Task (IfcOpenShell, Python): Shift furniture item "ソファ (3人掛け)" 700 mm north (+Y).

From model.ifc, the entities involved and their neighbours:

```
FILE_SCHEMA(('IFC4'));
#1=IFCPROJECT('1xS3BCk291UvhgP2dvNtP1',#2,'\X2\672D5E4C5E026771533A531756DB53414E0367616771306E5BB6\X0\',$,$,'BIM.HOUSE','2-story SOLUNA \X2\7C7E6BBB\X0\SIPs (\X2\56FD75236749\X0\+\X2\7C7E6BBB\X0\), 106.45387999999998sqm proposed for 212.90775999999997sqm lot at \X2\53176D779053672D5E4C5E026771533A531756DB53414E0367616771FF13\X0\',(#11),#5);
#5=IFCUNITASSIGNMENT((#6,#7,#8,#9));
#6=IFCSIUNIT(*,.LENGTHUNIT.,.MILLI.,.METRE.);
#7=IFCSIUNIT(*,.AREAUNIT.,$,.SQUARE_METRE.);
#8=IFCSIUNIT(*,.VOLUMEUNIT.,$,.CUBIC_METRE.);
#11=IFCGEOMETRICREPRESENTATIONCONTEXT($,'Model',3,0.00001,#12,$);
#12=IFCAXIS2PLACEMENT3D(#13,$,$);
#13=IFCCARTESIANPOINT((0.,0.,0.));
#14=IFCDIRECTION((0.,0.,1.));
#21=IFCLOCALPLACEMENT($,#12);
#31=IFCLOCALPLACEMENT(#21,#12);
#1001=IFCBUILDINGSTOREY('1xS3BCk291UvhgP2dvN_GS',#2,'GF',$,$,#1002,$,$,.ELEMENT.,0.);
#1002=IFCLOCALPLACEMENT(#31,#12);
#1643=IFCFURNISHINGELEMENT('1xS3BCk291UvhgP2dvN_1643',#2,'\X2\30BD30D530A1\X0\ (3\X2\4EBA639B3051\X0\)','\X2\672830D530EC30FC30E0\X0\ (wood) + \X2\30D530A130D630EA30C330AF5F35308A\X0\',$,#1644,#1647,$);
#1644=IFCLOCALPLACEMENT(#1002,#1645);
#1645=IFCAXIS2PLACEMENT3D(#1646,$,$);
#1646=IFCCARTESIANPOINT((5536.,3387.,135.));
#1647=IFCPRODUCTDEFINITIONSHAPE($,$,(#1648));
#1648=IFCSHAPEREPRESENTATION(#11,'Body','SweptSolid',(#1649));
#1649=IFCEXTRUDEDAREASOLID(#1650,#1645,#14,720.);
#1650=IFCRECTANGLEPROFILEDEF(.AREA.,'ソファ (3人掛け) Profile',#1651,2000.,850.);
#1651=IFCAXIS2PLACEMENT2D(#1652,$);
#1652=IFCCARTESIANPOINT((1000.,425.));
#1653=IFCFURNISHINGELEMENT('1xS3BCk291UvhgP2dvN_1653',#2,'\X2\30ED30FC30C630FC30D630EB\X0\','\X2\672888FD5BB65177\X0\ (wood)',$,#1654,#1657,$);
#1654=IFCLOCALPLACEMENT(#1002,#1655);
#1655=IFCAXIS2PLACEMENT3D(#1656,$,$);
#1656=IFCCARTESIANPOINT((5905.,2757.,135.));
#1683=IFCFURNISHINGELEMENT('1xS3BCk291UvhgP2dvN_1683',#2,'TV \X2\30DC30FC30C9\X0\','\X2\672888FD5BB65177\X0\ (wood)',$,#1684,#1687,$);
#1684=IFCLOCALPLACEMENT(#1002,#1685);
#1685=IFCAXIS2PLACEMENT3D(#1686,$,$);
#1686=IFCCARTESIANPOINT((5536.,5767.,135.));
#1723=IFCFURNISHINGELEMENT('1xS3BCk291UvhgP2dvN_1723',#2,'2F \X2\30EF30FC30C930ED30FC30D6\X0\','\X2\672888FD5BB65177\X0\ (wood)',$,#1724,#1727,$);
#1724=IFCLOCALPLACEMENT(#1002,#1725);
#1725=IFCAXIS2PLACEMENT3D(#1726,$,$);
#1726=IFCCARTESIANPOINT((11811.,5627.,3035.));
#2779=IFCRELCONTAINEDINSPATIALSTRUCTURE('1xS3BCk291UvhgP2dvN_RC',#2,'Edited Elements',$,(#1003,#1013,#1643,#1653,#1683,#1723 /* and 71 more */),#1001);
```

```python
import ifcopenshell
import ifcopenshell.api.geometry
import ifcopenshell.util.placement

model = ifcopenshell.open("model.ifc")

item = model.by_id(1643)
matrix = ifcopenshell.util.placement.get_local_placement(item.ObjectPlacement)
matrix[1, 3] += 700.0
ifcopenshell.api.geometry.edit_object_placement(model, product=item, matrix=matrix, is_si=False)

print(ifcopenshell.util.placement.get_local_placement(item.ObjectPlacement).round(3) + 0.0)

model.write("model_v2.ifc")
```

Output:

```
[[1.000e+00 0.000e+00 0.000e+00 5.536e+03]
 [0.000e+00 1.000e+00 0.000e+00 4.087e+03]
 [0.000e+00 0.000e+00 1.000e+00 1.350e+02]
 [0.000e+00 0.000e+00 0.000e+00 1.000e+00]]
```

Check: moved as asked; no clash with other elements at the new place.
